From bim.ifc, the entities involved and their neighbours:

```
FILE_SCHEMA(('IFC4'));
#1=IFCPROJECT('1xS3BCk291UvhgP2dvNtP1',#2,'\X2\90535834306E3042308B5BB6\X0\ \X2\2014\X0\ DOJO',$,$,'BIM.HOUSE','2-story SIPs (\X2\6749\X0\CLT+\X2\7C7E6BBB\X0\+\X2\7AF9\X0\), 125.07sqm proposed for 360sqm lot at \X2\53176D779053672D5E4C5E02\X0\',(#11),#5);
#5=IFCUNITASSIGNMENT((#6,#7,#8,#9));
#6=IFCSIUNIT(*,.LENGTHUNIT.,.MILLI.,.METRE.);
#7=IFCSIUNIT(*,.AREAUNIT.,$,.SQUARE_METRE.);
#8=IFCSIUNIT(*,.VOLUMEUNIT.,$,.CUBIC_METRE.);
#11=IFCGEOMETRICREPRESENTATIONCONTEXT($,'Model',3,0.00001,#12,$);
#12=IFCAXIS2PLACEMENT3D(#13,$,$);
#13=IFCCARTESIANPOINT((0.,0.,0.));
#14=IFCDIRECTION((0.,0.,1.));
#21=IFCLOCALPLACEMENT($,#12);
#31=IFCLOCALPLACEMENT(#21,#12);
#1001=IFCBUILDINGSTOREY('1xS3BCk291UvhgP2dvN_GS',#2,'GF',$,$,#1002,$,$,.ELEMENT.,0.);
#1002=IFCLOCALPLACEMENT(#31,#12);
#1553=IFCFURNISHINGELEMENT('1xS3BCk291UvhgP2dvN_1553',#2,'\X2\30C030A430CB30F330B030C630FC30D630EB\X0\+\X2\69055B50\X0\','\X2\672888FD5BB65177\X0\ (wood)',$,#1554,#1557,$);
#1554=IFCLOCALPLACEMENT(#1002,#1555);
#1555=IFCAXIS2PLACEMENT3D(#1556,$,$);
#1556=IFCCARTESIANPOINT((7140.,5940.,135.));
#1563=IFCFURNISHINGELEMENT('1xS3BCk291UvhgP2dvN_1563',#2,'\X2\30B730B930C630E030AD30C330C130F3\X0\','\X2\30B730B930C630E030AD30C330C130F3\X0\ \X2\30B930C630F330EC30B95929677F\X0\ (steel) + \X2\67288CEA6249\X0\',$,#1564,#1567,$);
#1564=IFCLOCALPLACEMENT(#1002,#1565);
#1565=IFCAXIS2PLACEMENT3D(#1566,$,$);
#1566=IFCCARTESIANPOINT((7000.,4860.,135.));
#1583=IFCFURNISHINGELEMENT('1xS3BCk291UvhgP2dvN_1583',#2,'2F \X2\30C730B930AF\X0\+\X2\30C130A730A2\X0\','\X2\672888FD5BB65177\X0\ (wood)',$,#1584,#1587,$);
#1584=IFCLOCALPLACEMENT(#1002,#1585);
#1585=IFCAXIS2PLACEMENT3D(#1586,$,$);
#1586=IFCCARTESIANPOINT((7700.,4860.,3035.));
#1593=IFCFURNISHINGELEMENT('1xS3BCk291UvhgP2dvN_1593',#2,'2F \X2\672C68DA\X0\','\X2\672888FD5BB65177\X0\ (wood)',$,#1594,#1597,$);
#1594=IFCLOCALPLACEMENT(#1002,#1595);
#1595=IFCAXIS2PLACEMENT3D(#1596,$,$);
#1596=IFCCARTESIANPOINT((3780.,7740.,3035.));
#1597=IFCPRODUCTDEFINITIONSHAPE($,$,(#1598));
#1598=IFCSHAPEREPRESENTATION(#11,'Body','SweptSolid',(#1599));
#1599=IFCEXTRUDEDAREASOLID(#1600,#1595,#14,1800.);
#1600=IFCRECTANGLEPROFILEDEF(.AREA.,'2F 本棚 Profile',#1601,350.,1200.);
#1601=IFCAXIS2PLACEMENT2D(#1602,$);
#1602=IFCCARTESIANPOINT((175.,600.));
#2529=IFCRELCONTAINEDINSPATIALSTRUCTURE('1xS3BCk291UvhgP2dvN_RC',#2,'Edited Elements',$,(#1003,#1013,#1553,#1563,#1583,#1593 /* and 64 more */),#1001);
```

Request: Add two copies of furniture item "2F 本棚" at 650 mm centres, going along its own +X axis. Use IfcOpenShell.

```python
import ifcopenshell
import ifcopenshell.api.geometry
import ifcopenshell.api.root
import ifcopenshell.util.element
import ifcopenshell.util.placement
import ifcopenshell.util.unit

model = ifcopenshell.open("bim.ifc")
unit_scale = ifcopenshell.util.unit.calculate_unit_scale(model)


def reuse_history(source, copy):
    """copy_class also copies each property set's owner history, people and application; keep the originals."""
    for rel in copy.IsDefinedBy:
        if rel.is_a("IfcRelDefinesByProperties") and (history := rel.RelatingPropertyDefinition.OwnerHistory):
            rel.RelatingPropertyDefinition.OwnerHistory = source.OwnerHistory
            ifcopenshell.util.element.remove_deep2(model, history)


source = model.by_guid("1xS3BCk291UvhgP2dvN_1593")
base = ifcopenshell.util.placement.get_local_placement(source.ObjectPlacement)
step = base[:3, 0] * 0.65 / unit_scale

for i in range(1, 3):
    copy = ifcopenshell.api.root.copy_class(model, product=source)
    copy.Representation = ifcopenshell.util.element.copy_deep(
        model, source.Representation, exclude=["IfcGeometricRepresentationContext", "IfcRepresentationMap"]
    )
    reuse_history(source, copy)
    matrix = base.copy()
    matrix[:3, 3] += i * step
    print("added at", matrix[:3, 3].round(3) + 0.0)
    ifcopenshell.api.geometry.edit_object_placement(model, product=copy, matrix=matrix, is_si=False)

model.write("bim_edited.ifc")
```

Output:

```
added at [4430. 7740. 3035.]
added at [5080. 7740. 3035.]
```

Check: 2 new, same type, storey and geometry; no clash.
